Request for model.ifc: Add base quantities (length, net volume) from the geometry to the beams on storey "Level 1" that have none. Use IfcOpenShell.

First a look at what the model holds.

```python
import ifcopenshell
import ifcopenshell.util.element
import ifcopenshell.util.unit

model = ifcopenshell.open("model.ifc")
print(model.schema)
for unit_type in ("LENGTHUNIT", "AREAUNIT", "VOLUMEUNIT"):
    print(unit_type, ifcopenshell.util.unit.calculate_unit_scale(model, unit_type))
storey = next(s for s in model.by_type("IfcBuildingStorey") if s.Name == "Level 1")
beams = [e for e in ifcopenshell.util.element.get_decomposition(storey) if e.is_a("IfcBeam")]
for e in sorted(beams, key=lambda e: e.id()):
    print(e.id(), e.is_a(), e.Name, list(ifcopenshell.util.element.get_psets(e, qtos_only=True)), sep=" | ")
```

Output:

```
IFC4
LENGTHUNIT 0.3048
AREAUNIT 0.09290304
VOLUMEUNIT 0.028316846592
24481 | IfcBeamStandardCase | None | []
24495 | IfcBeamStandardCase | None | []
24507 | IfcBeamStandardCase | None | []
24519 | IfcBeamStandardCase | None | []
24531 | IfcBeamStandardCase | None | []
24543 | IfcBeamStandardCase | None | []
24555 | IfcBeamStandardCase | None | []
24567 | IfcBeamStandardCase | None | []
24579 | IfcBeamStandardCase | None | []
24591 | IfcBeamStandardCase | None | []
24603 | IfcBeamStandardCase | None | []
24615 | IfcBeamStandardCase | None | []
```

```python
import ifcopenshell
import ifcopenshell.api.pset
import ifcopenshell.geom
import ifcopenshell.util.element
import ifcopenshell.util.shape
import ifcopenshell.util.unit

model = ifcopenshell.open("model.ifc")
unit_scale = ifcopenshell.util.unit.calculate_unit_scale(model)
volume_scale = ifcopenshell.util.unit.calculate_unit_scale(model, "VOLUMEUNIT")
settings = ifcopenshell.geom.settings()

storey = next(s for s in model.by_type("IfcBuildingStorey") if s.Name == "Level 1")
beams = [e for e in ifcopenshell.util.element.get_decomposition(storey) if e.is_a("IfcBeam")]

for e in sorted(beams, key=lambda e: e.id()):
    if ifcopenshell.util.element.get_psets(e, qtos_only=True, should_inherit=False):
        continue
    # Geometry comes back in metres, in the element's own axes.
    shape = ifcopenshell.geom.create_shape(settings, e)
    values = {
        "Length": ifcopenshell.util.shape.get_max_xyz(shape.geometry) / unit_scale,
        "NetVolume": ifcopenshell.util.shape.get_volume(shape.geometry) / volume_scale,
    }
    qto = ifcopenshell.api.pset.add_qto(model, product=e, name="Qto_BeamBaseQuantities")
    ifcopenshell.api.pset.edit_qto(model, qto=qto, properties=values)
    print(e.id(), {k: round(v, 3) for k, v in values.items()})

model.write("model_rev.ifc")
```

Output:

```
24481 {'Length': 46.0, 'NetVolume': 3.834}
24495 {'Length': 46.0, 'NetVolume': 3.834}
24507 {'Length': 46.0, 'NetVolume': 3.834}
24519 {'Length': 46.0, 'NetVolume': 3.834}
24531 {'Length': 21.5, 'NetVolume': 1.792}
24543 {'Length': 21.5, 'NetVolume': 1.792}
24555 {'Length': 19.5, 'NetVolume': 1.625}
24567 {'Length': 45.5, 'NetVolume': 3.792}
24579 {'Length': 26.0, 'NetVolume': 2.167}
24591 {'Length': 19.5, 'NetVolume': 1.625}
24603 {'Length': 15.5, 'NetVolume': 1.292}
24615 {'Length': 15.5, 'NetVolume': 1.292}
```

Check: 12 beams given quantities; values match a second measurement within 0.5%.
